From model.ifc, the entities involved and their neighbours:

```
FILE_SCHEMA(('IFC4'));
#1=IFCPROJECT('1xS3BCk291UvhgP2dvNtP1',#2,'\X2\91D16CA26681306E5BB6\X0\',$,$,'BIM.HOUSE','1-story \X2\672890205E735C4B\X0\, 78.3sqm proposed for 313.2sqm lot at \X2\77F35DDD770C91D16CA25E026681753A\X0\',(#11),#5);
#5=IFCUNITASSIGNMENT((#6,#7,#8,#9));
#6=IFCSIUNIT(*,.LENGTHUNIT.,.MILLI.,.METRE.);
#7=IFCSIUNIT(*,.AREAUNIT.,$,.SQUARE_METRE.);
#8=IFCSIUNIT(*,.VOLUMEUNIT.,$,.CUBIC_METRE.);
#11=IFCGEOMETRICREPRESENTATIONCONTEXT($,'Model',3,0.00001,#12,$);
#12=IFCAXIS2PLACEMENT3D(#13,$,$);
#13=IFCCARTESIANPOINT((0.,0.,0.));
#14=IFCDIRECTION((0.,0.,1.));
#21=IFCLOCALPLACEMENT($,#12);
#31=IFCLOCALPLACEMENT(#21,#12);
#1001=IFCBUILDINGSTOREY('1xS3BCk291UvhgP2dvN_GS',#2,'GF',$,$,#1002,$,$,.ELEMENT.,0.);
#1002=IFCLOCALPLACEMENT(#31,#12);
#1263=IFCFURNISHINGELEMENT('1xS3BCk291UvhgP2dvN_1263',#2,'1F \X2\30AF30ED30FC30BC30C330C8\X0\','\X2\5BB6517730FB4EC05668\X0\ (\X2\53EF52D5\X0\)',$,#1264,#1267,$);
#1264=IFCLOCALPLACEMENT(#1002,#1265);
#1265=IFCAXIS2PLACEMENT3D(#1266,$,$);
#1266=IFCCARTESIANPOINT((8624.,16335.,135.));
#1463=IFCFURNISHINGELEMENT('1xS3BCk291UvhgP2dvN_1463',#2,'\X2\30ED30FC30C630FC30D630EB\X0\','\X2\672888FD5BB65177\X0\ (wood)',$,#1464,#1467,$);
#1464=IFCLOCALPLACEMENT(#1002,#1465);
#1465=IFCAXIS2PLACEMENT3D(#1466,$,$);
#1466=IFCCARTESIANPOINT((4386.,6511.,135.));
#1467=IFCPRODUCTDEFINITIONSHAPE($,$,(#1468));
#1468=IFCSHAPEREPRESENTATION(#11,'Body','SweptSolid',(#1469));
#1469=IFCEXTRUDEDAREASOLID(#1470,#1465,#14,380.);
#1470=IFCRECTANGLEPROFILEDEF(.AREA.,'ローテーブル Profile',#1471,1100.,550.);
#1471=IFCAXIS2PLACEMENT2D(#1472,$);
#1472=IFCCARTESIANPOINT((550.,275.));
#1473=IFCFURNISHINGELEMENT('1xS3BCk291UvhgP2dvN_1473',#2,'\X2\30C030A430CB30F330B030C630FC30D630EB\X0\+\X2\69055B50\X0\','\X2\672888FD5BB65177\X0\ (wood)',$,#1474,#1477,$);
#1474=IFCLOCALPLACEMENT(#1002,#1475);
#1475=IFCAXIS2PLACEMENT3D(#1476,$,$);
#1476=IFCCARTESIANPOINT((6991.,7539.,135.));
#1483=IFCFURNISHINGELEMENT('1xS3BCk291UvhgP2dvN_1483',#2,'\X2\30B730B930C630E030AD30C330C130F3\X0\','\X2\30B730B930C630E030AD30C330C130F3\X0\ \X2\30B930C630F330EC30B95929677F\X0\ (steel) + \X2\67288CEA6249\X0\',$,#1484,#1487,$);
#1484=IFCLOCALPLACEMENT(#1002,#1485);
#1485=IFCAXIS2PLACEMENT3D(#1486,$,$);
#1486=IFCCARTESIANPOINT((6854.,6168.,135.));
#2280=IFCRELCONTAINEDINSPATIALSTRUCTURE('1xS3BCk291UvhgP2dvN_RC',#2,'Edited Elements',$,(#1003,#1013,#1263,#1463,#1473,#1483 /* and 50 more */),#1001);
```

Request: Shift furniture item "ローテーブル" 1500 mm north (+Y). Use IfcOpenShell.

```python
import ifcopenshell
import ifcopenshell.api.geometry
import ifcopenshell.util.placement
import ifcopenshell.util.unit

model = ifcopenshell.open("model.ifc")
unit_scale = ifcopenshell.util.unit.calculate_unit_scale(model)

item = model.by_guid("1xS3BCk291UvhgP2dvN_1463")
matrix = ifcopenshell.util.placement.get_local_placement(item.ObjectPlacement)
matrix[1, 3] += 1.5 / unit_scale
ifcopenshell.api.geometry.edit_object_placement(model, product=item, matrix=matrix, is_si=False)

print(ifcopenshell.util.placement.get_local_placement(item.ObjectPlacement).round(3) + 0.0)

model.write("model_edited.ifc")
```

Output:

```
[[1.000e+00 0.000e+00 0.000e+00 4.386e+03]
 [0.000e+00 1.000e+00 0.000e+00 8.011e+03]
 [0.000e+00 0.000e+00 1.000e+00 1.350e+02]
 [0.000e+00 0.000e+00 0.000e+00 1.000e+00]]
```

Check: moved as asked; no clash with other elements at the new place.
